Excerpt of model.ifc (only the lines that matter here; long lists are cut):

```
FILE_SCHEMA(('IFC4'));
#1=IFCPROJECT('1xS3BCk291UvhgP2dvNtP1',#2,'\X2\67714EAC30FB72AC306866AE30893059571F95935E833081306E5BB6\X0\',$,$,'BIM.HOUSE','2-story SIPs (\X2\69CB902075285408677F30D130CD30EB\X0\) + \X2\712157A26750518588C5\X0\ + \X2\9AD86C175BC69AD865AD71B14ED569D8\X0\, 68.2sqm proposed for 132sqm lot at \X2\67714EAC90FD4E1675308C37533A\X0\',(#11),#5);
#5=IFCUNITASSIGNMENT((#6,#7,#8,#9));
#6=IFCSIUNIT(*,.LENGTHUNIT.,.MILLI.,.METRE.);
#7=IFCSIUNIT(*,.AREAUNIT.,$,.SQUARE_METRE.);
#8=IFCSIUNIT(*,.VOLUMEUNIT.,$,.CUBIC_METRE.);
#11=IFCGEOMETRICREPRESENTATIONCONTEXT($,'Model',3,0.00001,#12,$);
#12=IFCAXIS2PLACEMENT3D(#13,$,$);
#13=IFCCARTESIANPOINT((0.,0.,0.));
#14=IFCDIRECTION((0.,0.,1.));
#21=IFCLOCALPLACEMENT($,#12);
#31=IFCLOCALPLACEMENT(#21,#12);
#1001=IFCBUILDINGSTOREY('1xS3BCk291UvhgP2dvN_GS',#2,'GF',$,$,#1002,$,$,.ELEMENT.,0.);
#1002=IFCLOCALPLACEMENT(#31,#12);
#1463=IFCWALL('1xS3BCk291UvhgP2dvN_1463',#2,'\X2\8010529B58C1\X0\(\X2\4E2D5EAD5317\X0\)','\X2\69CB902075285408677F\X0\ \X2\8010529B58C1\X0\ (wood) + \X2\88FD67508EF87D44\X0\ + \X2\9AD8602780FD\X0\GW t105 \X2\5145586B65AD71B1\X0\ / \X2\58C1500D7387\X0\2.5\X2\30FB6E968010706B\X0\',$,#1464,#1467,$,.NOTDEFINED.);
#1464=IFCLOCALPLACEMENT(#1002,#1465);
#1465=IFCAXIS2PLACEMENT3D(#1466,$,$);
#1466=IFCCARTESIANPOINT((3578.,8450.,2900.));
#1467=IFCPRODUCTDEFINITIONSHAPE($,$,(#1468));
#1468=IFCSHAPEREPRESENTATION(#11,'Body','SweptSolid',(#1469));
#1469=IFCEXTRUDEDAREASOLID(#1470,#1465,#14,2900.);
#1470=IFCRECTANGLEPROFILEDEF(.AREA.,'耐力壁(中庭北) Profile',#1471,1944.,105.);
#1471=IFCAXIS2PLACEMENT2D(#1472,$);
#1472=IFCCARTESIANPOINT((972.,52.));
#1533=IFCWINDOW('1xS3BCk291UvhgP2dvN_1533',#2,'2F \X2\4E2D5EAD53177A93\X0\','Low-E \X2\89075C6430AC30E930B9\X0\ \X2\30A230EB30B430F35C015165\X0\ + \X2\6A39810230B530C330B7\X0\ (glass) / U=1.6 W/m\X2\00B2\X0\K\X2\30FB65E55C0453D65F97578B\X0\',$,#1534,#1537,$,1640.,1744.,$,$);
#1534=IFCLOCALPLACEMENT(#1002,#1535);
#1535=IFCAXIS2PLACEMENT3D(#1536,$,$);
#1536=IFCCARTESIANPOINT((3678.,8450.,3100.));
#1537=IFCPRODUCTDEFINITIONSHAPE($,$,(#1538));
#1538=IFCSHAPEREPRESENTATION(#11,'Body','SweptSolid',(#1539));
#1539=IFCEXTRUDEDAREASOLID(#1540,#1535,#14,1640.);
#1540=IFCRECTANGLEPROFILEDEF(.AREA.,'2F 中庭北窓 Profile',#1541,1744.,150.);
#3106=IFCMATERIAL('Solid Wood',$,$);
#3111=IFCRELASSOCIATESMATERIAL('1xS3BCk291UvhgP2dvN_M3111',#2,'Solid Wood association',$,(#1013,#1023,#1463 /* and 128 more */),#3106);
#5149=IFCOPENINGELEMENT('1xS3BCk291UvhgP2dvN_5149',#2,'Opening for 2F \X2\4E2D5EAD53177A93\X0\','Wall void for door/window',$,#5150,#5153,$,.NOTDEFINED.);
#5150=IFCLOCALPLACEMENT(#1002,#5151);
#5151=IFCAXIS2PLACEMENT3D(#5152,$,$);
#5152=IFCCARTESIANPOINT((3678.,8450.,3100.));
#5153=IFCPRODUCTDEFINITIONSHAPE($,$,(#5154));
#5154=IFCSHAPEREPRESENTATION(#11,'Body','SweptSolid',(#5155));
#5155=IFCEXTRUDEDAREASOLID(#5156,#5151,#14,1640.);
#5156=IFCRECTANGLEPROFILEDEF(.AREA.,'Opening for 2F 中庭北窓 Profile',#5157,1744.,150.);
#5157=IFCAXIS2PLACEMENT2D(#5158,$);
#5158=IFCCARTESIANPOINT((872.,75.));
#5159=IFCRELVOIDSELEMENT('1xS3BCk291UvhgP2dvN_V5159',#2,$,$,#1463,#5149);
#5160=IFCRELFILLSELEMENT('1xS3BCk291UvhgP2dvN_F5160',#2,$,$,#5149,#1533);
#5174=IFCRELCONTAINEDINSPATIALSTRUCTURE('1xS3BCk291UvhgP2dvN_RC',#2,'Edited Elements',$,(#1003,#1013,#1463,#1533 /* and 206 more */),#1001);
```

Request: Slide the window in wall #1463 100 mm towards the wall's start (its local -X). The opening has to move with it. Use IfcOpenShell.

```python
import ifcopenshell
import ifcopenshell.api.geometry
import ifcopenshell.util.placement
import ifcopenshell.util.unit

model = ifcopenshell.open("model.ifc")
unit_scale = ifcopenshell.util.unit.calculate_unit_scale(model)

window = model.by_id(1533)
opening = window.FillsVoids[0].RelatingOpeningElement
wall = opening.VoidsElements[0].RelatingBuildingElement

wall_matrix = ifcopenshell.util.placement.get_local_placement(wall.ObjectPlacement)
shift = wall_matrix[:3, 0] * -0.1 / unit_scale
before = ifcopenshell.util.placement.get_local_placement(window.ObjectPlacement)[:3, 3].copy()

# The window is not placed relative to its opening, so move both.
for product in (opening, window):
    matrix = ifcopenshell.util.placement.get_local_placement(product.ObjectPlacement)
    matrix[:3, 3] += shift
    ifcopenshell.api.geometry.edit_object_placement(model, product=product, matrix=matrix, is_si=False)

after = ifcopenshell.util.placement.get_local_placement(window.ObjectPlacement)[:3, 3]
print("window moved by", (after - before).round(3) + 0.0)

model.write("model_edited.ifc")
```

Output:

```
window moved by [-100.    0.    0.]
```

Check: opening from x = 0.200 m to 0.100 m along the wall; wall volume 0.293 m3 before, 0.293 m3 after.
